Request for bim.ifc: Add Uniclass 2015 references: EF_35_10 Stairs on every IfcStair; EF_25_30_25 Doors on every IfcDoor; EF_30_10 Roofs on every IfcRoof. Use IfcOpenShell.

First a look at what the model holds.

```python
import ifcopenshell

model = ifcopenshell.open("bim.ifc")
print(model.schema)
print("classifications:", [c.Name for c in model.by_type("IfcClassification")])
for ifc_class in ("IfcDoor", "IfcRoof", "IfcStair", "IfcWall", "IfcWindow"):
    print(ifc_class, len(model.by_type(ifc_class)))
```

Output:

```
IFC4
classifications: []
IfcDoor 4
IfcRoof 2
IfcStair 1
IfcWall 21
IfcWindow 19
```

```python
import ifcopenshell
import ifcopenshell.api.classification

model = ifcopenshell.open("bim.ifc")

system = ifcopenshell.api.classification.add_classification(model, classification="Uniclass 2015")

codes = {
    "IfcStair": ("EF_35_10", "Stairs"),
    "IfcDoor": ("EF_25_30_25", "Doors"),
    "IfcRoof": ("EF_30_10", "Roofs"),
}
for ifc_class, (code, name) in codes.items():
    products = model.by_type(ifc_class)
    ifcopenshell.api.classification.add_reference(
        model, products=products, classification=system, identification=code, name=name
    )
    print(code, len(products))

model.write("bim_v2.ifc")
```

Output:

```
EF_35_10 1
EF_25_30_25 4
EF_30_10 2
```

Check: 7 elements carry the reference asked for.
